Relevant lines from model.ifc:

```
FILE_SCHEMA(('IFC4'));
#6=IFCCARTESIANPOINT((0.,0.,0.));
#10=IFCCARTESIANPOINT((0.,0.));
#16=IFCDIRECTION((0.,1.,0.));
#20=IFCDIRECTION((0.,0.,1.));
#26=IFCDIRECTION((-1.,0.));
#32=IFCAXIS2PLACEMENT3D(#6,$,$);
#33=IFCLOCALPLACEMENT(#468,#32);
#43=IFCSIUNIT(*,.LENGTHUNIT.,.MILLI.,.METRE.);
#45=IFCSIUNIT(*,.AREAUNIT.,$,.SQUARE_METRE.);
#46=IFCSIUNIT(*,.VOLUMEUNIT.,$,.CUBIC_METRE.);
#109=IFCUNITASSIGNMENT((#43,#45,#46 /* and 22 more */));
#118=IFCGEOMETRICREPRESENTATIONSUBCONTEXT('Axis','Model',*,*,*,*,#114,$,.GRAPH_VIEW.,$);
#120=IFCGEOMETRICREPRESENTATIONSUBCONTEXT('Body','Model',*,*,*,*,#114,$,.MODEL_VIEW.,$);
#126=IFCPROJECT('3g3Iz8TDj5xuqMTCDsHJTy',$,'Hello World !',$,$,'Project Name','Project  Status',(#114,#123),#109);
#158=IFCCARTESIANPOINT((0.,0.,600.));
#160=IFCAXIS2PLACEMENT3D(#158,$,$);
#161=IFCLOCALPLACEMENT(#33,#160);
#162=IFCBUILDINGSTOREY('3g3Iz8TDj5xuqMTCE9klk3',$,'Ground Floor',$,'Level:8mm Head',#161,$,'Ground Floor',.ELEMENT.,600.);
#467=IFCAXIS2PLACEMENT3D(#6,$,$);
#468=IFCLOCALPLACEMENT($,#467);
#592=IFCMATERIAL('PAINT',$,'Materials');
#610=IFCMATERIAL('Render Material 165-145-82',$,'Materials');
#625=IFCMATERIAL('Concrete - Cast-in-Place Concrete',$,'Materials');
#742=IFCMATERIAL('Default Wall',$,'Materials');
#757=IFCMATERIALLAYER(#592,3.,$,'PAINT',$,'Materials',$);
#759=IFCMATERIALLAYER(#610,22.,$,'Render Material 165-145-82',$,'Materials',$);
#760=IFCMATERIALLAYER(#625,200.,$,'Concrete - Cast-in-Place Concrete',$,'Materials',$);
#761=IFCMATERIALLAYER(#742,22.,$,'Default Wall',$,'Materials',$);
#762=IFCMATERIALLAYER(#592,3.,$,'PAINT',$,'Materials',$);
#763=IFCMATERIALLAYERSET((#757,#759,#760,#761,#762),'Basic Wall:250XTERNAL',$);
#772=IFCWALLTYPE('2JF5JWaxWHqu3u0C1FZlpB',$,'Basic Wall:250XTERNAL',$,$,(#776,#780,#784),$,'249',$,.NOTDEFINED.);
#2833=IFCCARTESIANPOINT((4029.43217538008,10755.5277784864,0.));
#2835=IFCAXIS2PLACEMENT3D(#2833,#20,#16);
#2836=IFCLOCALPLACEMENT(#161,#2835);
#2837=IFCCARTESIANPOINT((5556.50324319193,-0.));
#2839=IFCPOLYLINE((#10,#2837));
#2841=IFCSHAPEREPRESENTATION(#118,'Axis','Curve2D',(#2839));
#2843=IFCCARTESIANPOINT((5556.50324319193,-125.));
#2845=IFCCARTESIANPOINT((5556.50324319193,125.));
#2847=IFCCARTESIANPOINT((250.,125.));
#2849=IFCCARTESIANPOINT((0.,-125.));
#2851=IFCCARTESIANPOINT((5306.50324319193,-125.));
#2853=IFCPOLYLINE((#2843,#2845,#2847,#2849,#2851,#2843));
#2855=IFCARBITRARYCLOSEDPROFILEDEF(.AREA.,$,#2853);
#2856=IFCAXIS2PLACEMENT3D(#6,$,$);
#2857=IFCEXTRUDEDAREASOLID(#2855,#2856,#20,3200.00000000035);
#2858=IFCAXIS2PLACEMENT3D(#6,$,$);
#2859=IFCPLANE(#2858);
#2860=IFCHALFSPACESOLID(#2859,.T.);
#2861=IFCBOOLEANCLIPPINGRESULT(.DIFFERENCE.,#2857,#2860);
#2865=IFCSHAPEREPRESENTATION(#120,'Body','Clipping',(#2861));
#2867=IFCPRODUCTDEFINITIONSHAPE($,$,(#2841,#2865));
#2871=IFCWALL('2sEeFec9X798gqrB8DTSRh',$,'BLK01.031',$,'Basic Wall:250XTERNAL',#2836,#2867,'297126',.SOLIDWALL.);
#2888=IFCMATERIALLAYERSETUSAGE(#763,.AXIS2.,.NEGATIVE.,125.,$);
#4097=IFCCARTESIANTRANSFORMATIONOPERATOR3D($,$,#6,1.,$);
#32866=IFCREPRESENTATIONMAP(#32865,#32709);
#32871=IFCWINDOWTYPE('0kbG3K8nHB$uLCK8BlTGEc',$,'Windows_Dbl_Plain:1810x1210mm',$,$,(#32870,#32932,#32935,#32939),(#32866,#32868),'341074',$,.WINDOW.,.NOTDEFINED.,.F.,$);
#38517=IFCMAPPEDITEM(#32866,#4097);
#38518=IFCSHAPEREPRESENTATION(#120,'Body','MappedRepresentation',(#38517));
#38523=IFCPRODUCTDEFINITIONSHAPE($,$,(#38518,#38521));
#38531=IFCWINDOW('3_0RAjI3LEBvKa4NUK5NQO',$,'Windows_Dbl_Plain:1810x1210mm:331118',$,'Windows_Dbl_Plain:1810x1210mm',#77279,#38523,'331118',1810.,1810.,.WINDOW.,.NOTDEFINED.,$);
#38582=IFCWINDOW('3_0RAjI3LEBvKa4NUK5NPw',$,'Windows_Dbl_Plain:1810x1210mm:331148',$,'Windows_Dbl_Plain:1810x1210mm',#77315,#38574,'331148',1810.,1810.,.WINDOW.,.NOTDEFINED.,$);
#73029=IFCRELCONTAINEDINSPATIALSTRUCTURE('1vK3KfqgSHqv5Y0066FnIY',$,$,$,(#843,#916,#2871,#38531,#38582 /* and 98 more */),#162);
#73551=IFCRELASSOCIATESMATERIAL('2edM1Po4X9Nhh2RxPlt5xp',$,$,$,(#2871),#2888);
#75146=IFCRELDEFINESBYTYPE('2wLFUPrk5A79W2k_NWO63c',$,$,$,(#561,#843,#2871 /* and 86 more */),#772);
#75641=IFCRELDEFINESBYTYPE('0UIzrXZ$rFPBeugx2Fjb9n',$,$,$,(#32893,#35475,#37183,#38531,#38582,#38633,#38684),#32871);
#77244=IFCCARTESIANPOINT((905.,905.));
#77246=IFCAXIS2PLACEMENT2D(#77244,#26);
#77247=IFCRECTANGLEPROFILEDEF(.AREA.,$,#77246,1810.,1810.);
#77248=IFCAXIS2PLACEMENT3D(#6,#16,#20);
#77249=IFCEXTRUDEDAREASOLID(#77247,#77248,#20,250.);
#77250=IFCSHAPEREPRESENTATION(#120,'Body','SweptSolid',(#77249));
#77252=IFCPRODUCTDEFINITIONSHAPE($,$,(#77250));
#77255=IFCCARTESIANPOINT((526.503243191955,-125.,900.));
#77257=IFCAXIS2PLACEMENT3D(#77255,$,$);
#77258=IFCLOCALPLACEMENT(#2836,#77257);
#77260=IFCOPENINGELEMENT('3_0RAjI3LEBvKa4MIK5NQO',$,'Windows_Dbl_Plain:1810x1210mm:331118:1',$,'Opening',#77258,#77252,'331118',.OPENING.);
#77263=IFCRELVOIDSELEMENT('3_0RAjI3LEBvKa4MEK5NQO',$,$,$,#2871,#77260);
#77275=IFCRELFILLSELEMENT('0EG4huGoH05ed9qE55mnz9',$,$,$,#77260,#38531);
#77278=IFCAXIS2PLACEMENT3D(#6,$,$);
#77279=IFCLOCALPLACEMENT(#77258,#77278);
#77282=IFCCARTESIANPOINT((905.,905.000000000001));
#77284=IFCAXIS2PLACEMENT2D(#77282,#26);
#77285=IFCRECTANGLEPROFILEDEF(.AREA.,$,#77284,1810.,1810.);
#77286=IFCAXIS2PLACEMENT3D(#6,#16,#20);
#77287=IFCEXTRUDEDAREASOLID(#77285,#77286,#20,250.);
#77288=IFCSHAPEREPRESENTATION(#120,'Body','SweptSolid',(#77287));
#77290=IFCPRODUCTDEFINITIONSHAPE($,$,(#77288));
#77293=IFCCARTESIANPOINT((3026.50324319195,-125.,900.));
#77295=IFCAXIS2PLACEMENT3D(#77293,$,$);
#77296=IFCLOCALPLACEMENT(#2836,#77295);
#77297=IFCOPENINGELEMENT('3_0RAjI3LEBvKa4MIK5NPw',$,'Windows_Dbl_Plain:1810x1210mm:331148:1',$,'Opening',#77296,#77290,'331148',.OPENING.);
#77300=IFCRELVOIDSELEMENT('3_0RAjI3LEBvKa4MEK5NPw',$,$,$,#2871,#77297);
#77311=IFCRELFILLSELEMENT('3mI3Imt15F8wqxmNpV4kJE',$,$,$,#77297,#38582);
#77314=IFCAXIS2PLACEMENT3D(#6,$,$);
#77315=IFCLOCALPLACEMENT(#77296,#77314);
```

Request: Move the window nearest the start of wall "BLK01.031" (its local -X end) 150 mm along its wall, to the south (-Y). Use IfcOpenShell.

```python
import ifcopenshell
import ifcopenshell.api.geometry
import ifcopenshell.util.placement
import ifcopenshell.util.unit

model = ifcopenshell.open("model.ifc")
unit_scale = ifcopenshell.util.unit.calculate_unit_scale(model)

window = model.by_guid("3_0RAjI3LEBvKa4NUK5NQO")
opening = window.FillsVoids[0].RelatingOpeningElement
wall = opening.VoidsElements[0].RelatingBuildingElement

wall_matrix = ifcopenshell.util.placement.get_local_placement(wall.ObjectPlacement)
shift = wall_matrix[:3, 0] * -0.15 / unit_scale
before = ifcopenshell.util.placement.get_local_placement(window.ObjectPlacement)[:3, 3].copy()

# The window is placed relative to its opening, so it follows when the opening moves.
matrix = ifcopenshell.util.placement.get_local_placement(opening.ObjectPlacement)
matrix[:3, 3] += shift
ifcopenshell.api.geometry.edit_object_placement(
    model, product=opening, matrix=matrix, is_si=False, should_transform_children=True
)

after = ifcopenshell.util.placement.get_local_placement(window.ObjectPlacement)[:3, 3]
print("window moved by", (after - before).round(3) + 0.0)

model.write("model-out.ifc")
```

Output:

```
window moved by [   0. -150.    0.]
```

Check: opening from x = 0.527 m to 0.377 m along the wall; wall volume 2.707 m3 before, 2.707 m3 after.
